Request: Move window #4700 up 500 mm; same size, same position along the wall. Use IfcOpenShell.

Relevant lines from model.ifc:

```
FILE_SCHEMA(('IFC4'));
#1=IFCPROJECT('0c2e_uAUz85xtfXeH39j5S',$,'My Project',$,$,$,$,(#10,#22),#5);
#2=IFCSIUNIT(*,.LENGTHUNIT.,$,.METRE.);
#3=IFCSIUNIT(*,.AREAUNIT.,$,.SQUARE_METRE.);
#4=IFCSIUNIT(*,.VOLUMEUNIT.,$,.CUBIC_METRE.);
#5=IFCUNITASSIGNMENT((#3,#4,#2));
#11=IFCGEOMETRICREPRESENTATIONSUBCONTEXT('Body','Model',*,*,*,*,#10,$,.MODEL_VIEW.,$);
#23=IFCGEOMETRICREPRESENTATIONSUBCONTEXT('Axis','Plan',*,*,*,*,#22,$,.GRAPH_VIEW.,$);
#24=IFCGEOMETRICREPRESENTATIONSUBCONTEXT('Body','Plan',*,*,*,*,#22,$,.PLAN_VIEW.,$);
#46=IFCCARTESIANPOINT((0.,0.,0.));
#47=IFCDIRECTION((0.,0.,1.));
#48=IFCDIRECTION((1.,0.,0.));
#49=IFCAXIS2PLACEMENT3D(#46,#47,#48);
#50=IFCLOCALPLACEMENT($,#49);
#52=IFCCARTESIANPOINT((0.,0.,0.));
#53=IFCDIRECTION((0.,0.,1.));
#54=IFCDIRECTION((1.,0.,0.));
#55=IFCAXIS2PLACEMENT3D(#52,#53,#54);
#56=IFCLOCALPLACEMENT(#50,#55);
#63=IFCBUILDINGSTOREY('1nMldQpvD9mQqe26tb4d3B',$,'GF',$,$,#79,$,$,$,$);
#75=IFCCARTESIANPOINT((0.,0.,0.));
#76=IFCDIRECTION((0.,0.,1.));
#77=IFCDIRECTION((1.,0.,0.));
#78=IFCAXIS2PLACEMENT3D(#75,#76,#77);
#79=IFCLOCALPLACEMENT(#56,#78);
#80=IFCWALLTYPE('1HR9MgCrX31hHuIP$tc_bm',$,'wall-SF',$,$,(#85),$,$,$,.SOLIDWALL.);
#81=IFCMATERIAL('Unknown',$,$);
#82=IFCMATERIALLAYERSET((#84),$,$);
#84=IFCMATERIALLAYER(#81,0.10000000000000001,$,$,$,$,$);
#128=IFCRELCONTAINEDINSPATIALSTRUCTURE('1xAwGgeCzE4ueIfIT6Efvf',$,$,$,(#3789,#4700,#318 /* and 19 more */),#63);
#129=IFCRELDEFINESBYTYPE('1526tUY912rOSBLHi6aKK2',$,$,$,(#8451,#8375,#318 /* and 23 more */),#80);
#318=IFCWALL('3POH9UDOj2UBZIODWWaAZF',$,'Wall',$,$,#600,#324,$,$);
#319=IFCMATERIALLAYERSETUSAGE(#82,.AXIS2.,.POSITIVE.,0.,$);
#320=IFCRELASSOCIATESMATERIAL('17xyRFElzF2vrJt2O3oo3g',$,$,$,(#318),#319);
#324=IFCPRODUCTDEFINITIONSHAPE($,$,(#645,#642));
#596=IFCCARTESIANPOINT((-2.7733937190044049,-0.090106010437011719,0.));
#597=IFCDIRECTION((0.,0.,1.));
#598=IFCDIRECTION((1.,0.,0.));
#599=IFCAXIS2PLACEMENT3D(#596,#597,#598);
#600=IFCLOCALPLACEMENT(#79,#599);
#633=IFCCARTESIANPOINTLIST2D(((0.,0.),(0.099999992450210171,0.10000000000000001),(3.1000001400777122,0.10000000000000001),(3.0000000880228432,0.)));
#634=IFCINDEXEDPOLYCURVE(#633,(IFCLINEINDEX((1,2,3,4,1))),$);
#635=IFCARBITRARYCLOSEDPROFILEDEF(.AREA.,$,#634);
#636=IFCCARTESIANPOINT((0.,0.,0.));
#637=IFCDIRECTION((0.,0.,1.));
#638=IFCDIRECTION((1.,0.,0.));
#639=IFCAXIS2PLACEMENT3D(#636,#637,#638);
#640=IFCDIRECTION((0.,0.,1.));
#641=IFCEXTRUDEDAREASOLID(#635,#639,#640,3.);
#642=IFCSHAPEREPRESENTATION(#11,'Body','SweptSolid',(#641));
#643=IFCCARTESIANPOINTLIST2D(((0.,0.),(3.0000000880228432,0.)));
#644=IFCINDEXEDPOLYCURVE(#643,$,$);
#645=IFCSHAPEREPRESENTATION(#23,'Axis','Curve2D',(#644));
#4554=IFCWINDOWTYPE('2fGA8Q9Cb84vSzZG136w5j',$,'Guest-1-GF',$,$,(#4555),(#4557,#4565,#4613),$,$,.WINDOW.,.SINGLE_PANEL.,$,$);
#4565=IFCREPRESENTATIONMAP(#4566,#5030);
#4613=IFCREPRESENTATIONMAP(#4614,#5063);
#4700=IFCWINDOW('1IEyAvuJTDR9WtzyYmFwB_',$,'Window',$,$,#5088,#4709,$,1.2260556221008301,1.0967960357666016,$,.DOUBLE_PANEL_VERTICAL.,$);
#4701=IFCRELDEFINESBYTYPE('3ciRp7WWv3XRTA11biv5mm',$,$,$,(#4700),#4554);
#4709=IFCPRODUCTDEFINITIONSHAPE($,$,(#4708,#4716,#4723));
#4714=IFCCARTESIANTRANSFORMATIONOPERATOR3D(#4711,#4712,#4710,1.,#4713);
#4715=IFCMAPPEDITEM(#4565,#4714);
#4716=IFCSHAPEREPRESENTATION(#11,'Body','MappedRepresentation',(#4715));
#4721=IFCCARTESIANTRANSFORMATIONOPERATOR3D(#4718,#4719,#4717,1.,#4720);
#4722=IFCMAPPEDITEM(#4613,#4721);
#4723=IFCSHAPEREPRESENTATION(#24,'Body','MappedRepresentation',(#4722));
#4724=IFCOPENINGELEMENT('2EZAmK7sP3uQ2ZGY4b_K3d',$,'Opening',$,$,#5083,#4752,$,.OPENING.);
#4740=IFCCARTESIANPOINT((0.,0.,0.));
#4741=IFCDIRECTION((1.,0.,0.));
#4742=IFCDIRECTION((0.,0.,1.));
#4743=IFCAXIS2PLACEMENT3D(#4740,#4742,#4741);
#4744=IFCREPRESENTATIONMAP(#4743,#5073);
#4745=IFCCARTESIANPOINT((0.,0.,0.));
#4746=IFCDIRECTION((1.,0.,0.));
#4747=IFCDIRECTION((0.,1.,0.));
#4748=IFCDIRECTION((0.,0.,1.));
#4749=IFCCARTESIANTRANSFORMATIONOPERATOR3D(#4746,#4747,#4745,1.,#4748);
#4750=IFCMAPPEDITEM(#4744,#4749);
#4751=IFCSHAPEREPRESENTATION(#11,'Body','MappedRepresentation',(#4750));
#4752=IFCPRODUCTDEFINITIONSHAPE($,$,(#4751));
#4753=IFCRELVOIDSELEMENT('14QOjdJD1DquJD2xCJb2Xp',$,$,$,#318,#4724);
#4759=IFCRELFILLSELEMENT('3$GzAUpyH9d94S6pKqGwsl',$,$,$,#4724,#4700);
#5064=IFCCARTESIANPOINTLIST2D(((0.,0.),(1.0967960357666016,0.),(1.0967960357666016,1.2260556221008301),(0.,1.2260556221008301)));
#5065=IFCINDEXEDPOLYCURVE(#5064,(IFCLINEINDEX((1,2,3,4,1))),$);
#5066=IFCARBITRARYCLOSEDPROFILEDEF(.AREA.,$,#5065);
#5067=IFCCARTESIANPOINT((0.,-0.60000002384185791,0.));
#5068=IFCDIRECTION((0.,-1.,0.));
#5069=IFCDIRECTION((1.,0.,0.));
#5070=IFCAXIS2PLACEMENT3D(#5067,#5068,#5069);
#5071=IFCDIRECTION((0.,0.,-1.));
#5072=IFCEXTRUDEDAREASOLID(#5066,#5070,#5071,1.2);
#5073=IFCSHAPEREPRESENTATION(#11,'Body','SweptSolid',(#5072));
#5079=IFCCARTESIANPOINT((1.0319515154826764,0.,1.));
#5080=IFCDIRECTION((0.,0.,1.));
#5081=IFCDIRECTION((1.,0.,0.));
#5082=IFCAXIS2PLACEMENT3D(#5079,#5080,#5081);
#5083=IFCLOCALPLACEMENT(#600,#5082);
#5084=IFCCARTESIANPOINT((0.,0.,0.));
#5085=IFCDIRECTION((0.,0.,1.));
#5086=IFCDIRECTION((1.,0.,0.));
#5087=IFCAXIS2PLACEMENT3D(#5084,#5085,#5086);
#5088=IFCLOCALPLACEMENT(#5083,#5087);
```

```python
import numpy as np
import ifcopenshell
import ifcopenshell.api.geometry
import ifcopenshell.util.placement
import ifcopenshell.util.unit

model = ifcopenshell.open("model.ifc")
unit_scale = ifcopenshell.util.unit.calculate_unit_scale(model)

window = model.by_guid("1IEyAvuJTDR9WtzyYmFwB_")
opening = window.FillsVoids[0].RelatingOpeningElement
dz = 0.5

shift = np.array([0.0, 0.0, dz])
# The window is placed relative to its opening, so it follows when the opening moves.
matrix = ifcopenshell.util.placement.get_local_placement(opening.ObjectPlacement)
matrix[:3, 3] += shift
ifcopenshell.api.geometry.edit_object_placement(
    model, product=opening, matrix=matrix, is_si=False, should_transform_children=True
)

print(f"moved by {dz * unit_scale:+.3f} m")

model.write("model_v2.ifc")
```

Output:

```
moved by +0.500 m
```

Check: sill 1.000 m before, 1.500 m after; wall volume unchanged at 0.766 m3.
